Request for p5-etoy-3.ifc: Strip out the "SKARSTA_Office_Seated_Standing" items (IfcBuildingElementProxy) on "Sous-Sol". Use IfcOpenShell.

First a look at what the model holds.

```python
import ifcopenshell
import ifcopenshell.util.element

model = ifcopenshell.open("p5-etoy-3.ifc")
print(model.schema)
storey = next(s for s in model.by_type("IfcBuildingStorey") if s.Name == "Sous-Sol")
proxies = [e for e in ifcopenshell.util.element.get_decomposition(storey) if e.is_a("IfcBuildingElementProxy")]
seen = {}
for e in proxies:
    element_type = ifcopenshell.util.element.get_type(e)
    name = element_type.Name if element_type not in (None, e) else None
    seen[name] = seen.get(name, 0) + 1
for name, count in sorted(seen.items(), key=str):
    print(count, "x", name)
```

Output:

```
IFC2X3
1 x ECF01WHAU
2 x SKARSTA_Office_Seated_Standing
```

```python
import ifcopenshell
import ifcopenshell.api.root
import ifcopenshell.util.element

model = ifcopenshell.open("p5-etoy-3.ifc")

storey = next(s for s in model.by_type("IfcBuildingStorey") if s.Name == "Sous-Sol")
proxies = [e for e in ifcopenshell.util.element.get_decomposition(storey) if e.is_a("IfcBuildingElementProxy")]
targets = [e for e in proxies if (t := ifcopenshell.util.element.get_type(e)) not in (None, e) and t.Name == "SKARSTA_Office_Seated_Standing"]

for e in targets:
    ifcopenshell.api.root.remove_product(model, product=e)
print(len(targets), "removed")

model.write("p5-etoy-3_updated.ifc")
```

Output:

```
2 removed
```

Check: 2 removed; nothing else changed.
